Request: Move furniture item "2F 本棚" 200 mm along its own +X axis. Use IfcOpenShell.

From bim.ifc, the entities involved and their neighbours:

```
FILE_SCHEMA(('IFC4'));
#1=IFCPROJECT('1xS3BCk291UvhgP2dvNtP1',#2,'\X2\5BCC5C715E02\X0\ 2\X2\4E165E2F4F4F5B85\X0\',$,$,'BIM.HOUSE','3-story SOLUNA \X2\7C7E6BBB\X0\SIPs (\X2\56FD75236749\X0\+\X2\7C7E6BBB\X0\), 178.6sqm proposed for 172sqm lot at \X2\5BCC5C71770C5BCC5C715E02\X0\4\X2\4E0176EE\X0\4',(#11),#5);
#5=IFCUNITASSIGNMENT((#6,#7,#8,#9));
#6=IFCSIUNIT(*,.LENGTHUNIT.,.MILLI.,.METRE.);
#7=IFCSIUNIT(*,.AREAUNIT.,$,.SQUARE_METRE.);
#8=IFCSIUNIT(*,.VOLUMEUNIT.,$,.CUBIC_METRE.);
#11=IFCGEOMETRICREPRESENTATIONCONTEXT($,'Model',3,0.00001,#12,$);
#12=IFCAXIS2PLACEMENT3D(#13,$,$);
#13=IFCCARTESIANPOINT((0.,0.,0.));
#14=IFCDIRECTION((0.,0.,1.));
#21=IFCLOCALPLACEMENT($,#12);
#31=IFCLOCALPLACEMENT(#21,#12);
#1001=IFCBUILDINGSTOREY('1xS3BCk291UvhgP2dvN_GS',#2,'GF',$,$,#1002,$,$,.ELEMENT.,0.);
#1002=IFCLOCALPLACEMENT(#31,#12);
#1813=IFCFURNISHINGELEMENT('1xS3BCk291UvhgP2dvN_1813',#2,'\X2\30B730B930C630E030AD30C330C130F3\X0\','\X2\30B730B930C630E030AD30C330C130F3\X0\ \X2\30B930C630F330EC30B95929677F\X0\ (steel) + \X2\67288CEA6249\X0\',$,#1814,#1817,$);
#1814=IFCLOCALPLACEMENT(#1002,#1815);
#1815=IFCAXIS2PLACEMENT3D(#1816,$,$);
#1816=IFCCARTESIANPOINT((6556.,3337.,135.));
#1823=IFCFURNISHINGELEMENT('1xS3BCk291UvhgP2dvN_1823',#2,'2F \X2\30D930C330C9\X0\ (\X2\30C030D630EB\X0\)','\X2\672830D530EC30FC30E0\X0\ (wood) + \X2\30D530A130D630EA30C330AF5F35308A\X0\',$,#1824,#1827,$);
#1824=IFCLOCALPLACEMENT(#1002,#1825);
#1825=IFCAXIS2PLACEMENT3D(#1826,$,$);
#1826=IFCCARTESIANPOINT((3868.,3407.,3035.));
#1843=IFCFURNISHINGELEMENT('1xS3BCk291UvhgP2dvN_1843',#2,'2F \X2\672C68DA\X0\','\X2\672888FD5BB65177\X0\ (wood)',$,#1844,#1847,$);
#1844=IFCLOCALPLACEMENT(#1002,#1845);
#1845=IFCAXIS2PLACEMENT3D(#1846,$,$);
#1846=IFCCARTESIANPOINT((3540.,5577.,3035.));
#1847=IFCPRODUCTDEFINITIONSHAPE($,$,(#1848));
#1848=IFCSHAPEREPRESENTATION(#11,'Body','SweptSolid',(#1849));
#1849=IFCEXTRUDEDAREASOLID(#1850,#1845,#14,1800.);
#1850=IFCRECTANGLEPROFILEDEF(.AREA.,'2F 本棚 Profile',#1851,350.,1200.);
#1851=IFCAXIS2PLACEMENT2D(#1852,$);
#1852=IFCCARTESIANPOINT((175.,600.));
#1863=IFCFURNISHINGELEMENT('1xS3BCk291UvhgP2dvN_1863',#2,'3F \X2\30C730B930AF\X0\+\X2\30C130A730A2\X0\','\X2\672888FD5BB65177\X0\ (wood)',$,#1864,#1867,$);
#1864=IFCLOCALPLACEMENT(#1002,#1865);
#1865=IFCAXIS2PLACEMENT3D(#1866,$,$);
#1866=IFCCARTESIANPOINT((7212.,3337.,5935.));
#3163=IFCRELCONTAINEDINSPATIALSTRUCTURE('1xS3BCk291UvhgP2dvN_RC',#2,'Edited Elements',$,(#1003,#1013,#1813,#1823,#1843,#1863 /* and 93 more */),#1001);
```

```python
import ifcopenshell
import ifcopenshell.api.geometry
import ifcopenshell.util.placement
import ifcopenshell.util.unit

model = ifcopenshell.open("bim.ifc")
unit_scale = ifcopenshell.util.unit.calculate_unit_scale(model)

item = model.by_guid("1xS3BCk291UvhgP2dvN_1843")
matrix = ifcopenshell.util.placement.get_local_placement(item.ObjectPlacement)
matrix[:3, 3] += matrix[:3, 0] * 0.2 / unit_scale
ifcopenshell.api.geometry.edit_object_placement(model, product=item, matrix=matrix, is_si=False)

print(ifcopenshell.util.placement.get_local_placement(item.ObjectPlacement).round(3) + 0.0)

model.write("bim-out.ifc")
```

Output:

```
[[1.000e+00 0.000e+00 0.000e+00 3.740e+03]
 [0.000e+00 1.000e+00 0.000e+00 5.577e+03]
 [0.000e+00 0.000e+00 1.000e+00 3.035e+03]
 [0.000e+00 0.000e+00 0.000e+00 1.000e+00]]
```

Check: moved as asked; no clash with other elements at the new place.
